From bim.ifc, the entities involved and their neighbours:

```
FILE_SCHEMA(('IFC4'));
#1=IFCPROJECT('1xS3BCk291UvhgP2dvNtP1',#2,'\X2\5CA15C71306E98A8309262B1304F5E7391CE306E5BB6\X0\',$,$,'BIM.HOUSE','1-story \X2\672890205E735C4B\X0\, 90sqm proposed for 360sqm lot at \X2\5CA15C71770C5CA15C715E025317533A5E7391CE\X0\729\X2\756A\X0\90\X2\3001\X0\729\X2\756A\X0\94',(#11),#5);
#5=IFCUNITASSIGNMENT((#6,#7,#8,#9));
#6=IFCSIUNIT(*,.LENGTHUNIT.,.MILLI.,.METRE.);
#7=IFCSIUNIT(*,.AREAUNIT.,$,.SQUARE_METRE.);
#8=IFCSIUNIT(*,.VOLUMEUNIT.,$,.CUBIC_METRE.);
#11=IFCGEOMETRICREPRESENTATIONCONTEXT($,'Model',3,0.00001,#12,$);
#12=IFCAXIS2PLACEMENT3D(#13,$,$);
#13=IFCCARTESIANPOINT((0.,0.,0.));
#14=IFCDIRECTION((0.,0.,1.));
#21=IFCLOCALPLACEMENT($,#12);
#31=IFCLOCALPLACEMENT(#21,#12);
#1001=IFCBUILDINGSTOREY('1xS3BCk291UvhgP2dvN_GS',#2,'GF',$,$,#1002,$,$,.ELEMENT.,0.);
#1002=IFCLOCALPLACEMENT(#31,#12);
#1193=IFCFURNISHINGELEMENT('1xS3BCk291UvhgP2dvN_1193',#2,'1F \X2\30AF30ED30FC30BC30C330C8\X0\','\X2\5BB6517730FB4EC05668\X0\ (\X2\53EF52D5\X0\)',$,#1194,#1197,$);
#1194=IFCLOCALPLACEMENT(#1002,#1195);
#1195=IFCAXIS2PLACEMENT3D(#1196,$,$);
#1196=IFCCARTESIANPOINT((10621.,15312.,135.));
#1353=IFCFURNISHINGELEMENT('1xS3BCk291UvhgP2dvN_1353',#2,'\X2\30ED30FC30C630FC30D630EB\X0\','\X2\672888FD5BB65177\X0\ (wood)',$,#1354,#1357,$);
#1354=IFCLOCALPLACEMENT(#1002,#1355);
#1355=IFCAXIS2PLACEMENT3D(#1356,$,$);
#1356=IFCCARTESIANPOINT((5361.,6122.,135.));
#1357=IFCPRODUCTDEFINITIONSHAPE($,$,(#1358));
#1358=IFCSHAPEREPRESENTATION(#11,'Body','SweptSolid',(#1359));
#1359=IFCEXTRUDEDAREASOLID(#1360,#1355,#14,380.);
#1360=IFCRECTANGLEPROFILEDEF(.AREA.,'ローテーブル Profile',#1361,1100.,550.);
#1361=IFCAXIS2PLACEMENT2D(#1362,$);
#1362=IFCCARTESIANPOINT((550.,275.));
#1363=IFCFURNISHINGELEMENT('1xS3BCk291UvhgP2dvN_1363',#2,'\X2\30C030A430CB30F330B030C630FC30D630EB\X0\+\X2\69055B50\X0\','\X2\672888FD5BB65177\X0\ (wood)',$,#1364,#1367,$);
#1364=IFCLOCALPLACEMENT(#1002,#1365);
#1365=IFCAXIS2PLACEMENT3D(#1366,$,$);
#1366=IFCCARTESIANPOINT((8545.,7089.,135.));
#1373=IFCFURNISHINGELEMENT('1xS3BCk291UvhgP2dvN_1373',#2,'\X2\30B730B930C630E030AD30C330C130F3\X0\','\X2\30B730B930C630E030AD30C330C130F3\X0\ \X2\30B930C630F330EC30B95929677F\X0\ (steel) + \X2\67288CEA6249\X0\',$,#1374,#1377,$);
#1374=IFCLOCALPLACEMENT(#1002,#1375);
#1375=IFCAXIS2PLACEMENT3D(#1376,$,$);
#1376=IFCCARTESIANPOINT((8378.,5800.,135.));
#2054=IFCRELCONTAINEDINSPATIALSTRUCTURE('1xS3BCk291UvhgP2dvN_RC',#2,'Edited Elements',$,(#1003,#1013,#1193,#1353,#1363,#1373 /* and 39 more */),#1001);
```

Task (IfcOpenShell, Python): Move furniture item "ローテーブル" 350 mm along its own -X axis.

```python
import ifcopenshell
import ifcopenshell.api.geometry
import ifcopenshell.util.placement
import ifcopenshell.util.unit

model = ifcopenshell.open("bim.ifc")
unit_scale = ifcopenshell.util.unit.calculate_unit_scale(model)

item = model.by_guid("1xS3BCk291UvhgP2dvN_1353")
matrix = ifcopenshell.util.placement.get_local_placement(item.ObjectPlacement)
matrix[:3, 3] -= matrix[:3, 0] * 0.35 / unit_scale
ifcopenshell.api.geometry.edit_object_placement(model, product=item, matrix=matrix, is_si=False)

print(ifcopenshell.util.placement.get_local_placement(item.ObjectPlacement).round(3) + 0.0)

model.write("bim_edited.ifc")
```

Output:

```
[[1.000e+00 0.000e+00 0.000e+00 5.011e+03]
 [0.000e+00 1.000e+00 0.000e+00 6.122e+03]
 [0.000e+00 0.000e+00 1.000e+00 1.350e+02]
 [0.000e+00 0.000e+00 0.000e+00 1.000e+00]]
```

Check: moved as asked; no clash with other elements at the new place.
